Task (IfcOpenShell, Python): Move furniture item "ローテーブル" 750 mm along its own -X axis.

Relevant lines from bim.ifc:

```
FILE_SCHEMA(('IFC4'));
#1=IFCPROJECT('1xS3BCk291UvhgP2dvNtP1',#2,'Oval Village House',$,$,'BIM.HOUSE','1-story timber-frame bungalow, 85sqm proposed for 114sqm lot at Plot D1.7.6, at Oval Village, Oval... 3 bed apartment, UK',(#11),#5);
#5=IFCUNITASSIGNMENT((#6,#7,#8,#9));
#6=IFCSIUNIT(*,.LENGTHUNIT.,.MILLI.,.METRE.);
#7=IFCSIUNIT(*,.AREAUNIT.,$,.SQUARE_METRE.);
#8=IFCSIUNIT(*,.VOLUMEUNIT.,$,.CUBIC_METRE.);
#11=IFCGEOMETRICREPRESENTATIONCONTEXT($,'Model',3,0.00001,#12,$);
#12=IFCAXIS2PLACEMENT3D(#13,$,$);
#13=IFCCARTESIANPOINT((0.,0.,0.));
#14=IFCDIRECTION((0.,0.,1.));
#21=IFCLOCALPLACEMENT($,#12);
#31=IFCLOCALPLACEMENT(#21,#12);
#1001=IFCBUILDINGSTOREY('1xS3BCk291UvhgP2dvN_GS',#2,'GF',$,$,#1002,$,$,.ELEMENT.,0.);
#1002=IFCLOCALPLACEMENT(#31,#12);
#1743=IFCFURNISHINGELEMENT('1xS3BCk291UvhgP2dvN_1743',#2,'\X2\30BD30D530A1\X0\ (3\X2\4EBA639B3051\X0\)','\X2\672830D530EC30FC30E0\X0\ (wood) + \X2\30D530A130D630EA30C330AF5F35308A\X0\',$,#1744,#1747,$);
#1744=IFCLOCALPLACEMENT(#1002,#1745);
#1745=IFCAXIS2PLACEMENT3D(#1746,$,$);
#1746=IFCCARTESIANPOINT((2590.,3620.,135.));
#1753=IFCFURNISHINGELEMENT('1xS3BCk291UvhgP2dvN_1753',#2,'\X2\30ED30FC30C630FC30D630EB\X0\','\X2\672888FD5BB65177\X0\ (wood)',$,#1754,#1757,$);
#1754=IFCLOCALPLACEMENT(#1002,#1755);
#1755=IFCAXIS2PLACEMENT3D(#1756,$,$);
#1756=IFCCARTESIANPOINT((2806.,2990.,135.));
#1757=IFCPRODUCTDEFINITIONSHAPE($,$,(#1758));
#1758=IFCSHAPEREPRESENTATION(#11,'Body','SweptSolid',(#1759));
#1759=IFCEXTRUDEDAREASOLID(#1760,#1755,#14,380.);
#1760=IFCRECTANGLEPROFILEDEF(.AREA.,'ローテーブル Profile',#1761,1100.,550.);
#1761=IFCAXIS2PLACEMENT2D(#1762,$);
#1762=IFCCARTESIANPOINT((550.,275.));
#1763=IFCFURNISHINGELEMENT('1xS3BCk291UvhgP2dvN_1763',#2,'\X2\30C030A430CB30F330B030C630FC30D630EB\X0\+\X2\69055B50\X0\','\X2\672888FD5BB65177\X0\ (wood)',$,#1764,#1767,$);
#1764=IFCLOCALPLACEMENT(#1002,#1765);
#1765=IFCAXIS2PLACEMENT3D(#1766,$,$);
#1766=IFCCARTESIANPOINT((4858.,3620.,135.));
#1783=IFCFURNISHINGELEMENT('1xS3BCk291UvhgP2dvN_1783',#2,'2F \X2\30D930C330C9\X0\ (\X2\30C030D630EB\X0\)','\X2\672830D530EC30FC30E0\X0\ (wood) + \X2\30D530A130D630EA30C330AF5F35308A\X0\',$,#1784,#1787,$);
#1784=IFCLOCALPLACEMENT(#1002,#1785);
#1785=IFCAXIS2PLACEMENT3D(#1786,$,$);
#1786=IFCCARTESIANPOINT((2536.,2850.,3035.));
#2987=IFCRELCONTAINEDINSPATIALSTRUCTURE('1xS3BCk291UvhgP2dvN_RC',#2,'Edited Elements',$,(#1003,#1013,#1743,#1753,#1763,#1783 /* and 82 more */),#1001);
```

```python
import ifcopenshell
import ifcopenshell.api.geometry
import ifcopenshell.util.placement
import ifcopenshell.util.unit

model = ifcopenshell.open("bim.ifc")
unit_scale = ifcopenshell.util.unit.calculate_unit_scale(model)

item = model.by_guid("1xS3BCk291UvhgP2dvN_1753")
matrix = ifcopenshell.util.placement.get_local_placement(item.ObjectPlacement)
matrix[:3, 3] -= matrix[:3, 0] * 0.75 / unit_scale
ifcopenshell.api.geometry.edit_object_placement(model, product=item, matrix=matrix, is_si=False)

print(ifcopenshell.util.placement.get_local_placement(item.ObjectPlacement).round(3) + 0.0)

model.write("bim_rev.ifc")
```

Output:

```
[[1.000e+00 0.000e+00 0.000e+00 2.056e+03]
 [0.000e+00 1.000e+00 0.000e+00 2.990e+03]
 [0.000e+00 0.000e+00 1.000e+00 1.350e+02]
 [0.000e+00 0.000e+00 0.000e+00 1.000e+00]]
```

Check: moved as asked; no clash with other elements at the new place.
